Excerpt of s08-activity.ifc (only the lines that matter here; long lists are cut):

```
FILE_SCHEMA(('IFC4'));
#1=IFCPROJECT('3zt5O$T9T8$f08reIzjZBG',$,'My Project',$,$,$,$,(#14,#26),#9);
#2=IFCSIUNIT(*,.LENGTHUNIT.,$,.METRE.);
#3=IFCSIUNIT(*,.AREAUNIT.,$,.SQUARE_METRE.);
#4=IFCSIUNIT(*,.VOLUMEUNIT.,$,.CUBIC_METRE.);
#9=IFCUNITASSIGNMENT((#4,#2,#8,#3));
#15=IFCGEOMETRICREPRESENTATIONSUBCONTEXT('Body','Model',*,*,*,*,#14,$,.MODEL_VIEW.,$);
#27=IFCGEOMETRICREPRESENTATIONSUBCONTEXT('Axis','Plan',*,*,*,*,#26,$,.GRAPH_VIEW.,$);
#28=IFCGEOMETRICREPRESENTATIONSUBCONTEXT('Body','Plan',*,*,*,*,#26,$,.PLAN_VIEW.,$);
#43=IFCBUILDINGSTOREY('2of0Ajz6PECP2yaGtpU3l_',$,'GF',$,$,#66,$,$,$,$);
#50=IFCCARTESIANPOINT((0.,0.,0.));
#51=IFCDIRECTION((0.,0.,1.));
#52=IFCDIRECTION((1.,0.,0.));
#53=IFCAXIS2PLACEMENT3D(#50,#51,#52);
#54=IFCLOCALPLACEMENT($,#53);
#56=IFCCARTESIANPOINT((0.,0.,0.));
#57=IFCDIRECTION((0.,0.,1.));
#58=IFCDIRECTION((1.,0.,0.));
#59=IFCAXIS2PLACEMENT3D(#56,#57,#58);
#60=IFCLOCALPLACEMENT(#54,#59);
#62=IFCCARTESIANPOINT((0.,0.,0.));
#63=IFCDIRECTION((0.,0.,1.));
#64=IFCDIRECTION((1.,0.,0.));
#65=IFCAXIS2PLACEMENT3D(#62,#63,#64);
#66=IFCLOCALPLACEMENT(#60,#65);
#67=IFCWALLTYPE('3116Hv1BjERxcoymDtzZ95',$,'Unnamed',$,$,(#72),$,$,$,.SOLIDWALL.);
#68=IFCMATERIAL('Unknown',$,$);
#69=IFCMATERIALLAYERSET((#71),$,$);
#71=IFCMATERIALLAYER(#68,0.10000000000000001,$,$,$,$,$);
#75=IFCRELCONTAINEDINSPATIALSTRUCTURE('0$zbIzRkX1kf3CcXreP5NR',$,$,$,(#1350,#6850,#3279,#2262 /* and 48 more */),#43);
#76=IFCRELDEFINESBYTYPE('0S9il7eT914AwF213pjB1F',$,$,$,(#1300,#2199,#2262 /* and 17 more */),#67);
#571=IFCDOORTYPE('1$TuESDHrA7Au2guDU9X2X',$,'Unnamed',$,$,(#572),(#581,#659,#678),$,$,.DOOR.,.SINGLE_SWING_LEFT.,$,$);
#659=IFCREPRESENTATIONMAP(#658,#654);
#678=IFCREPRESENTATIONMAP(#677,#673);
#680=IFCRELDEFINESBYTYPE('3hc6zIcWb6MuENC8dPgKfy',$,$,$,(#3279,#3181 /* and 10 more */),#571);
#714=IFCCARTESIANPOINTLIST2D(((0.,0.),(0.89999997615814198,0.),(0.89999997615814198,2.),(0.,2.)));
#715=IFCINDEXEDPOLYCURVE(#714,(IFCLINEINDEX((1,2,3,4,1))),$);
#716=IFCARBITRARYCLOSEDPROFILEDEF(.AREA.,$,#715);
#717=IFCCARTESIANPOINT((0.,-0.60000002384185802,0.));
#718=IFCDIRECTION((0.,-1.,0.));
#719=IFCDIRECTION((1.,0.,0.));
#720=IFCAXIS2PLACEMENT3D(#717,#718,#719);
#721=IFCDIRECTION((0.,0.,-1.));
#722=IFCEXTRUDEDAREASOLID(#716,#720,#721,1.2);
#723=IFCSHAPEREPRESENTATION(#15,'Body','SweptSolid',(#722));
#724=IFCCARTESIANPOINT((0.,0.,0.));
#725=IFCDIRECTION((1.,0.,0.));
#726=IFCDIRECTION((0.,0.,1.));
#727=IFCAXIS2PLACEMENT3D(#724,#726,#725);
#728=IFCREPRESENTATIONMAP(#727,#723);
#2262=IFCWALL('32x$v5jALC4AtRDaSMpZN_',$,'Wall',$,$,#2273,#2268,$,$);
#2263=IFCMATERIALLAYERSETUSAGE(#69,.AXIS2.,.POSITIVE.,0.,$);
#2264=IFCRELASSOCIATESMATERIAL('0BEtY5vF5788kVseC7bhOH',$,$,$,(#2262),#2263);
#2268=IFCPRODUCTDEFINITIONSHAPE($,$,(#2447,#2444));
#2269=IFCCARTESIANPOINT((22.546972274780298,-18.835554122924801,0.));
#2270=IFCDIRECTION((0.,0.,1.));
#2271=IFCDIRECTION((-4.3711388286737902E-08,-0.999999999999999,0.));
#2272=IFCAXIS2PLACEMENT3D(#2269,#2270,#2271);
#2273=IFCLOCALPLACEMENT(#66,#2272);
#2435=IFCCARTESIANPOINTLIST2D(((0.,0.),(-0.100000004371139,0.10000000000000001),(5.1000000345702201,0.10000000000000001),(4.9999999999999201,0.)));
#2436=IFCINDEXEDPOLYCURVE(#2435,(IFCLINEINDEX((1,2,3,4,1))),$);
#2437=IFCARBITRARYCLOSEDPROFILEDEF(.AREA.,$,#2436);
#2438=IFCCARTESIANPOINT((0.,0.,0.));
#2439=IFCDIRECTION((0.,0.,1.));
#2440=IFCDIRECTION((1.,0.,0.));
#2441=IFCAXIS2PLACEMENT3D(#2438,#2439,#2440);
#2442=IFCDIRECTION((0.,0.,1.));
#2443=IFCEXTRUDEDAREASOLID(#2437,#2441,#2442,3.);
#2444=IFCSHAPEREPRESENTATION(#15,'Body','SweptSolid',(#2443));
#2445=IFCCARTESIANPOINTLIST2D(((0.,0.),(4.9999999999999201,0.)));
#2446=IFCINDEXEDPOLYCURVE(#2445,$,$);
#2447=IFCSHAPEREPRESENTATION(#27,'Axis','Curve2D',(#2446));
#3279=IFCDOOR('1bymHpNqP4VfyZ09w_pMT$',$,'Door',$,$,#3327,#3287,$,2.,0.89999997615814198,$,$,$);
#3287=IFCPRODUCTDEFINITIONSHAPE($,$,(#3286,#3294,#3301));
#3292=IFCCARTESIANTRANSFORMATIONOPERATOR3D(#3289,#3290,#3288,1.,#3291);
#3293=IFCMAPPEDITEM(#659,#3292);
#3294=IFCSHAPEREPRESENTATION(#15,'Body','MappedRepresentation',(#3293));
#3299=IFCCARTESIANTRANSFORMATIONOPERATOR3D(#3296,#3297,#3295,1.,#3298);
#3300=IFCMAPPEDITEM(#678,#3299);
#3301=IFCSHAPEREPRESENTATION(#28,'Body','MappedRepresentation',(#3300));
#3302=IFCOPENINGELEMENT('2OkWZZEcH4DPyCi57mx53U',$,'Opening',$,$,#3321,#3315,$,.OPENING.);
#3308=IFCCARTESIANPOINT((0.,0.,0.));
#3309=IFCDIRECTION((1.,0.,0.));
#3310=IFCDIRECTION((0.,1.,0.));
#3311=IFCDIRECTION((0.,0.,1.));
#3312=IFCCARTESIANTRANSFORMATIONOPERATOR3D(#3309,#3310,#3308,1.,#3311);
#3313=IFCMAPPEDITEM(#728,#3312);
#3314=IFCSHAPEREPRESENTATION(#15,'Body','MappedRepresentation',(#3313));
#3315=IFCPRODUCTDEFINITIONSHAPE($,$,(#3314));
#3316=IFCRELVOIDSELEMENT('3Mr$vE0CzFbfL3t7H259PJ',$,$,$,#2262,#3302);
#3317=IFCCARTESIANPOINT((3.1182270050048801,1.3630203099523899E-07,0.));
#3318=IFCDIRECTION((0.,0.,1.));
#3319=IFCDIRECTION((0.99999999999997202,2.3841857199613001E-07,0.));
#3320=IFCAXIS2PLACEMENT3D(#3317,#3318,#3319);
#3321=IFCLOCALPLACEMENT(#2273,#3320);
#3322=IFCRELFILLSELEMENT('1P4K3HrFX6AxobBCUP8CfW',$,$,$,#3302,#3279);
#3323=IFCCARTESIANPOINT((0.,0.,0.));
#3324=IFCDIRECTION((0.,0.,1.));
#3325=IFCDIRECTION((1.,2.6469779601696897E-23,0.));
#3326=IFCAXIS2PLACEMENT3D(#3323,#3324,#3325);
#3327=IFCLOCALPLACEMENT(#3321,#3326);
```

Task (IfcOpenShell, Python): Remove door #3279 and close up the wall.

```python
import ifcopenshell
import ifcopenshell.api.feature
import ifcopenshell.api.root
import ifcopenshell.geom
import ifcopenshell.util.shape

model = ifcopenshell.open("s08-activity.ifc")
settings = ifcopenshell.geom.settings()


def volume(element):
    """Net volume in cubic metres, openings subtracted."""
    shape = ifcopenshell.geom.create_shape(settings, element)
    return ifcopenshell.util.shape.get_volume(shape.geometry)


door = model.by_id(3279)
opening = door.FillsVoids[0].RelatingOpeningElement
wall = opening.VoidsElements[0].RelatingBuildingElement
before = volume(wall)

ifcopenshell.api.root.remove_product(model, product=door)
ifcopenshell.api.feature.remove_feature(model, feature=opening)

after = volume(wall)

print(f"wall volume {before:.3f} -> {after:.3f} m3")

model.write("s08-activity_updated.ifc")
```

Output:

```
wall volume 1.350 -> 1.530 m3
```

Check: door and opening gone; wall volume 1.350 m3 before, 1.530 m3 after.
